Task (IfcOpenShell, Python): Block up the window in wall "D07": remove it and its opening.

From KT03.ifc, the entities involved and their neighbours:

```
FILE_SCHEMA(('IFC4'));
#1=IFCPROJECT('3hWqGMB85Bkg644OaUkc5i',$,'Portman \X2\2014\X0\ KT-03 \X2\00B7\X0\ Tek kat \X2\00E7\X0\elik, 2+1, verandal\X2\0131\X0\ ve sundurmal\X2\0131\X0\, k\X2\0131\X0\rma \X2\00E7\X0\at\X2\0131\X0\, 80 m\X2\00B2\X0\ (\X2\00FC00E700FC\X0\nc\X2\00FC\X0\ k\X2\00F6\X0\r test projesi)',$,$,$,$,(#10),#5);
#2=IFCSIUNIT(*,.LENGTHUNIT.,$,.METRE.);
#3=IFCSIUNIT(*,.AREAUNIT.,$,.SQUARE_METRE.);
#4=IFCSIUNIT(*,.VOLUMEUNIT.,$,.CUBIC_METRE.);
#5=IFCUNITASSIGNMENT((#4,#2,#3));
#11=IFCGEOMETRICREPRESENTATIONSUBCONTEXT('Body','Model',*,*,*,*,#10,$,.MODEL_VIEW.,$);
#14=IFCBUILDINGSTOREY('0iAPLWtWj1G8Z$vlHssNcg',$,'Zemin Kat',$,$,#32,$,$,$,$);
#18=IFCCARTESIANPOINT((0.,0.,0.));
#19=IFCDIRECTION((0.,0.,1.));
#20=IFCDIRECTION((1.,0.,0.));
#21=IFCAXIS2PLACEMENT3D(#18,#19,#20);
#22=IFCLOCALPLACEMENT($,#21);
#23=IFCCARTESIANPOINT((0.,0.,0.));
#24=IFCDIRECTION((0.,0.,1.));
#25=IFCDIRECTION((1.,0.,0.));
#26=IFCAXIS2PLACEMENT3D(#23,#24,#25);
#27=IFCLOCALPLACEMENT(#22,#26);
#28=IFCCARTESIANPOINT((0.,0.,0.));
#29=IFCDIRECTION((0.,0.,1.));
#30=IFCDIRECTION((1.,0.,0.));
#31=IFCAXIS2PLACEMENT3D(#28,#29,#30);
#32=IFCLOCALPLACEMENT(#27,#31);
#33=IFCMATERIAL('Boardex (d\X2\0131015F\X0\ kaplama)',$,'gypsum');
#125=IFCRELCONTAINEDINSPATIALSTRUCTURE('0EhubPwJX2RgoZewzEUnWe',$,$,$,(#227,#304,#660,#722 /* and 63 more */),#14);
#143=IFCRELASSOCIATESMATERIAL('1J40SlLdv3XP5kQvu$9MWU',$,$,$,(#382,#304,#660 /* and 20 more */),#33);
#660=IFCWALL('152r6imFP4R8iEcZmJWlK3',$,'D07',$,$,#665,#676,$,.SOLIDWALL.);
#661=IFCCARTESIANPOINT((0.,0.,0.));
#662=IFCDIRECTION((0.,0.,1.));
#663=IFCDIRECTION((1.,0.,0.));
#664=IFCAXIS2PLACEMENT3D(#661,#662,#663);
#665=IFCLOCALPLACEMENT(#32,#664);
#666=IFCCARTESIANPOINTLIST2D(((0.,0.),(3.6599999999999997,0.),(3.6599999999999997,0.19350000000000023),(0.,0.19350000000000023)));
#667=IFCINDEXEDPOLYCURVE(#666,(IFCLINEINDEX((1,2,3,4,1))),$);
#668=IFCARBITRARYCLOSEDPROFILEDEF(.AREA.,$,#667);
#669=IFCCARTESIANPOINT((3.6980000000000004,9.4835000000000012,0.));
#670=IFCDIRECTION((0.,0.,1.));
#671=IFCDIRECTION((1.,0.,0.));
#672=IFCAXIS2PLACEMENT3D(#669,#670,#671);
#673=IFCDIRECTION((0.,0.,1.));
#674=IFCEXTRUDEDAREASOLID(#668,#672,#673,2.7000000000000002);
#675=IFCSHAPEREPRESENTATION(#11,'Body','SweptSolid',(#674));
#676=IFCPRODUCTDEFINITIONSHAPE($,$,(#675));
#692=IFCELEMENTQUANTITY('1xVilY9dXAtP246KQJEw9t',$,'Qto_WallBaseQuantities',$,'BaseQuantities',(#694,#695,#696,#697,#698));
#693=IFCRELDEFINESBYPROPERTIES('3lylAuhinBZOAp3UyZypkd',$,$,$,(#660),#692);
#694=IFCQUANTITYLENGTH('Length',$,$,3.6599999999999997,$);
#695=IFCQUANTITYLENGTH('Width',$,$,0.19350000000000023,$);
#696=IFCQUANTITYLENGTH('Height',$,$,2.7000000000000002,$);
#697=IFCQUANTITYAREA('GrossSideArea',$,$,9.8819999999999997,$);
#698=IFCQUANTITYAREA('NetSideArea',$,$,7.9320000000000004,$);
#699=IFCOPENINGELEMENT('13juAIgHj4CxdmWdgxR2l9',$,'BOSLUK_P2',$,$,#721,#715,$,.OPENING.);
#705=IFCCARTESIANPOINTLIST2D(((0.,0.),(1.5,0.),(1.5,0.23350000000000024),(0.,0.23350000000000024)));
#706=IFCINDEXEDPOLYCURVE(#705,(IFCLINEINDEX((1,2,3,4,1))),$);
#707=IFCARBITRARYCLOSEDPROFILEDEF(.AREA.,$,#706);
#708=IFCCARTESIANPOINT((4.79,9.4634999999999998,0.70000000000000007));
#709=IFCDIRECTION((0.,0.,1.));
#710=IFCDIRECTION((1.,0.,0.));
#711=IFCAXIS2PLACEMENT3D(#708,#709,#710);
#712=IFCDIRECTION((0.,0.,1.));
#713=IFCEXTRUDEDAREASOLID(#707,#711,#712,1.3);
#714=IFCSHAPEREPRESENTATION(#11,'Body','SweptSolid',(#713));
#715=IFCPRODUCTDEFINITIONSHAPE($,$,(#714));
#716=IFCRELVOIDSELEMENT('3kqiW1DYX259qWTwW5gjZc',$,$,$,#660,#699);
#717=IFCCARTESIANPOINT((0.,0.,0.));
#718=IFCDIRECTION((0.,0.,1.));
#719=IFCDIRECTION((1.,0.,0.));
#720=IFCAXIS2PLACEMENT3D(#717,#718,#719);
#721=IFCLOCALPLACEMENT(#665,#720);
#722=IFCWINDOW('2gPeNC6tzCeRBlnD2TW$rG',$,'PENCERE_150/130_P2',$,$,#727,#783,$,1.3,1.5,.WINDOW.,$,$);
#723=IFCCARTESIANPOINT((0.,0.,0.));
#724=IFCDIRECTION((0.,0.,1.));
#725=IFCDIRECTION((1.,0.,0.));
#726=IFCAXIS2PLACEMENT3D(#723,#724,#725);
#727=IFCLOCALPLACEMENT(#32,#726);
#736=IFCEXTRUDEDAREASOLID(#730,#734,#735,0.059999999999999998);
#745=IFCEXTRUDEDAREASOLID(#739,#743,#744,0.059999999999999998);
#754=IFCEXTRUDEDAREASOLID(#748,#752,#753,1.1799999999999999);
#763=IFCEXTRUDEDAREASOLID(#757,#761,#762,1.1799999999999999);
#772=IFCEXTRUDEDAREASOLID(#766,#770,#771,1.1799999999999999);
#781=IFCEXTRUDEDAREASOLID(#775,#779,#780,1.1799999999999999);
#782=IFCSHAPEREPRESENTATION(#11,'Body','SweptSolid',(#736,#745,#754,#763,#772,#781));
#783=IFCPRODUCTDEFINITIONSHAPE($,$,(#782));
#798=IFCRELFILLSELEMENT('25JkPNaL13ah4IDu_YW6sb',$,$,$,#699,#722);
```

```python
import ifcopenshell
import ifcopenshell.api.feature
import ifcopenshell.api.pset
import ifcopenshell.api.root
import ifcopenshell.geom
import ifcopenshell.util.element
import ifcopenshell.util.shape
import ifcopenshell.util.unit

model = ifcopenshell.open("KT03.ifc")
area_scale = ifcopenshell.util.unit.calculate_unit_scale(model, "AREAUNIT")
settings = ifcopenshell.geom.settings()


def volume(element):
    """Net volume in cubic metres, openings subtracted."""
    shape = ifcopenshell.geom.create_shape(settings, element)
    return ifcopenshell.util.shape.get_volume(shape.geometry)


window = model.by_guid("2gPeNC6tzCeRBlnD2TW$rG")
opening = window.FillsVoids[0].RelatingOpeningElement
wall = opening.VoidsElements[0].RelatingBuildingElement
before = volume(wall)

ifcopenshell.api.root.remove_product(model, product=window)
ifcopenshell.api.feature.remove_feature(model, feature=opening)

after = volume(wall)
thickness = 0.1935  # wall thickness in metres

# Update the wall's stored quantities.
qto = model.by_id(ifcopenshell.util.element.get_pset(wall, "Qto_WallBaseQuantities", should_inherit=False)["id"])
ifcopenshell.api.pset.edit_qto(model, qto=qto, properties={"NetSideArea": after / thickness / area_scale})

print(f"wall volume {before:.3f} -> {after:.3f} m3")

model.write("KT03_v2.ifc")
```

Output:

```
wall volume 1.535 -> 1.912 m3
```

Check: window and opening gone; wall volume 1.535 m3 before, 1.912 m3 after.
